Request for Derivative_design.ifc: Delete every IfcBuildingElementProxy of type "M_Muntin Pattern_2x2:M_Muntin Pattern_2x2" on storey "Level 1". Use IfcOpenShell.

First a look at what the model holds.

```python
import ifcopenshell
import ifcopenshell.util.element

model = ifcopenshell.open("Derivative_design.ifc")
print(model.schema)
storey = next(s for s in model.by_type("IfcBuildingStorey") if s.Name == "Level 1")
proxies = [e for e in ifcopenshell.util.element.get_decomposition(storey) if e.is_a("IfcBuildingElementProxy")]
seen = {}
for e in proxies:
    element_type = ifcopenshell.util.element.get_type(e)
    name = element_type.Name if element_type not in (None, e) else None
    seen[name] = seen.get(name, 0) + 1
for name, count in sorted(seen.items(), key=str):
    print(count, "x", name)
```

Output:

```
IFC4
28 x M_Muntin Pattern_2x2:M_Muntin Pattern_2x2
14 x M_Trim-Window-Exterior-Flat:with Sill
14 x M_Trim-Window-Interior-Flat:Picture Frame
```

```python
import ifcopenshell
import ifcopenshell.api.root
import ifcopenshell.util.element

model = ifcopenshell.open("Derivative_design.ifc")

storey = next(s for s in model.by_type("IfcBuildingStorey") if s.Name == "Level 1")
proxies = [e for e in ifcopenshell.util.element.get_decomposition(storey) if e.is_a("IfcBuildingElementProxy")]
targets = [e for e in proxies if (t := ifcopenshell.util.element.get_type(e)) not in (None, e) and t.Name == "M_Muntin Pattern_2x2:M_Muntin Pattern_2x2"]

for e in targets:
    ifcopenshell.api.root.remove_product(model, product=e)
print(len(targets), "removed")

model.write("Derivative_design_v2.ifc")
```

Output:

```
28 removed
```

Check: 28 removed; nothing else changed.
